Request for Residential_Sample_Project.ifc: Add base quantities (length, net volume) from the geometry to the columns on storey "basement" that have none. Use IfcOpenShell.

First a look at what the model holds.

```python
import ifcopenshell
import ifcopenshell.util.element
import ifcopenshell.util.unit

model = ifcopenshell.open("Residential_Sample_Project.ifc")
print(model.schema)
for unit_type in ("LENGTHUNIT", "AREAUNIT", "VOLUMEUNIT"):
    print(unit_type, ifcopenshell.util.unit.calculate_unit_scale(model, unit_type))
storey = next(s for s in model.by_type("IfcBuildingStorey") if s.Name == "basement")
columns = [e for e in ifcopenshell.util.element.get_decomposition(storey) if e.is_a("IfcColumn")]
for e in sorted(columns, key=lambda e: e.id()):
    print(e.id(), e.is_a(), e.Name, list(ifcopenshell.util.element.get_psets(e, qtos_only=True)), sep=" | ")
```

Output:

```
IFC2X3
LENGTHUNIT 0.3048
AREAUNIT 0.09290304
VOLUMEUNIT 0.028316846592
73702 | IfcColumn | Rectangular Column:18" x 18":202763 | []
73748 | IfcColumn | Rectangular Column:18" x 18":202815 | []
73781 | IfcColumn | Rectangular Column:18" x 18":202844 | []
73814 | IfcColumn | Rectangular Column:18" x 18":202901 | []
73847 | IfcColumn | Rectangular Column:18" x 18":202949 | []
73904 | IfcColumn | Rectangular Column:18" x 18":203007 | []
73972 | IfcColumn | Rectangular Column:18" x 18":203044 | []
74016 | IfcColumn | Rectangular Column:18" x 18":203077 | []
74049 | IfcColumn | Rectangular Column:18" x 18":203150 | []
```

```python
import ifcopenshell
import ifcopenshell.api.pset
import ifcopenshell.geom
import ifcopenshell.util.element
import ifcopenshell.util.shape
import ifcopenshell.util.unit

model = ifcopenshell.open("Residential_Sample_Project.ifc")
unit_scale = ifcopenshell.util.unit.calculate_unit_scale(model)
volume_scale = ifcopenshell.util.unit.calculate_unit_scale(model, "VOLUMEUNIT")
settings = ifcopenshell.geom.settings()

storey = next(s for s in model.by_type("IfcBuildingStorey") if s.Name == "basement")
columns = [e for e in ifcopenshell.util.element.get_decomposition(storey) if e.is_a("IfcColumn")]

for e in sorted(columns, key=lambda e: e.id()):
    if ifcopenshell.util.element.get_psets(e, qtos_only=True, should_inherit=False):
        continue
    # Geometry comes back in metres, in the element's own axes.
    shape = ifcopenshell.geom.create_shape(settings, e)
    values = {
        "Length": ifcopenshell.util.shape.get_z(shape.geometry) / unit_scale,
        "NetVolume": ifcopenshell.util.shape.get_volume(shape.geometry) / volume_scale,
    }
    qto = ifcopenshell.api.pset.add_qto(model, product=e, name="BaseQuantities")
    ifcopenshell.api.pset.edit_qto(model, qto=qto, properties=values)
    print(e.id(), {k: round(v, 3) for k, v in values.items()})

model.write("Residential_Sample_Project_edited.ifc")
```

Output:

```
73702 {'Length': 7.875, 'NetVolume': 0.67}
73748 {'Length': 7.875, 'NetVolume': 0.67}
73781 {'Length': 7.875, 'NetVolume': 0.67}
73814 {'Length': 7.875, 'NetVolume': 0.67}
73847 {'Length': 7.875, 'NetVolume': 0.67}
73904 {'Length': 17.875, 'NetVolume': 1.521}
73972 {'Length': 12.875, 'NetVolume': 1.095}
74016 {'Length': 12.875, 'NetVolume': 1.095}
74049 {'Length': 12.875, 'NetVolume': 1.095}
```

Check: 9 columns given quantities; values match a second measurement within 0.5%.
